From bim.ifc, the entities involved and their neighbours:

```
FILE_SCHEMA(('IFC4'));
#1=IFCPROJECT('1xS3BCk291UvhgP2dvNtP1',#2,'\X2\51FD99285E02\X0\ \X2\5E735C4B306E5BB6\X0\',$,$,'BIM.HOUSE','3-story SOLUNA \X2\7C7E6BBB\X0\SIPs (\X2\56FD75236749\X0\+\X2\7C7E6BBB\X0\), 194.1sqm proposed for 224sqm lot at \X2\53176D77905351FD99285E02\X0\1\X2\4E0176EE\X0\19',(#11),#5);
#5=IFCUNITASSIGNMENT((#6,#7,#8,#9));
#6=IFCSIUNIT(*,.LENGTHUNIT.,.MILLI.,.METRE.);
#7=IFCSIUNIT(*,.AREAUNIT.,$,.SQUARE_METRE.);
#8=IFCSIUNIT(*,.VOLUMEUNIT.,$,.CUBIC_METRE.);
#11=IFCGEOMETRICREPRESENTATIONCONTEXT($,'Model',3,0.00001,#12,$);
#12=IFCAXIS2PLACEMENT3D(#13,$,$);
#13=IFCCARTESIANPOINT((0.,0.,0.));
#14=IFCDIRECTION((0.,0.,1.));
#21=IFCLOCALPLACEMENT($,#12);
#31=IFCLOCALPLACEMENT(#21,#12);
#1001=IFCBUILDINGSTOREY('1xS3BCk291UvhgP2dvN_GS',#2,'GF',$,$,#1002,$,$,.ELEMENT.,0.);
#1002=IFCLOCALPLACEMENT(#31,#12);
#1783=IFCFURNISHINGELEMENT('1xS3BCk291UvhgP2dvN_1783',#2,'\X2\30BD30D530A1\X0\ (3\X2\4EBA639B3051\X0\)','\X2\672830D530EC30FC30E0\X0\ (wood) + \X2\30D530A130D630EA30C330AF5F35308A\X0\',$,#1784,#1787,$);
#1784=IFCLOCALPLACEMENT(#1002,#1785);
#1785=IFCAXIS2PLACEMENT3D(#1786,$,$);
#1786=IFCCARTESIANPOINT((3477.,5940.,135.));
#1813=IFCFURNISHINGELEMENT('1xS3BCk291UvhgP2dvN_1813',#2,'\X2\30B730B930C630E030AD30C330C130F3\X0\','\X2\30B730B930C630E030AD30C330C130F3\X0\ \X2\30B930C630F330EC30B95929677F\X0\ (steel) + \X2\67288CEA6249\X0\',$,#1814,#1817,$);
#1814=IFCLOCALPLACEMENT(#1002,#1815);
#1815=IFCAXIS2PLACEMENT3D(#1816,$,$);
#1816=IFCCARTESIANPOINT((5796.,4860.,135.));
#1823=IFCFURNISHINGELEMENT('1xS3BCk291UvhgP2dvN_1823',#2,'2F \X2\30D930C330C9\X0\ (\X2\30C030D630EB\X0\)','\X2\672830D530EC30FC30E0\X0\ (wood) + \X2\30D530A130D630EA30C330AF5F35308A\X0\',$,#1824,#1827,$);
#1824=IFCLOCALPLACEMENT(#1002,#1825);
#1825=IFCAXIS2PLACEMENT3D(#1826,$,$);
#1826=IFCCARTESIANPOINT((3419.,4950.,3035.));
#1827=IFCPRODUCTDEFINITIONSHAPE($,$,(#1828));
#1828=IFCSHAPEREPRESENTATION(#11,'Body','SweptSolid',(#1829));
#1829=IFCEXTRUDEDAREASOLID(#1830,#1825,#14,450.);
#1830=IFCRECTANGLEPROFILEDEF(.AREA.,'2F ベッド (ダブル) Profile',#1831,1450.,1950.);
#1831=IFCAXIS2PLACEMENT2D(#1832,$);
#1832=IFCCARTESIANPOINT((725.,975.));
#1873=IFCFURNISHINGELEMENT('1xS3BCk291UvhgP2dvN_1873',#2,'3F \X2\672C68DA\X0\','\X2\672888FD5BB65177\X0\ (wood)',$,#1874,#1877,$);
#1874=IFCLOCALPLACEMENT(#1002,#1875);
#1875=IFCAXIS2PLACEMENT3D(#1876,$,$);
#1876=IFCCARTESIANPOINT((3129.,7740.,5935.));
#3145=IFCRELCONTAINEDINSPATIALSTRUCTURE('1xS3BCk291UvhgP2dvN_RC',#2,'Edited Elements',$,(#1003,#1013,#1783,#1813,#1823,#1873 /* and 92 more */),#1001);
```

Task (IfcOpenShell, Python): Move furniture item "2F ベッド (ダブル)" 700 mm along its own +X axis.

```python
import ifcopenshell
import ifcopenshell.api.geometry
import ifcopenshell.util.placement

model = ifcopenshell.open("bim.ifc")

item = model.by_id(1823)
matrix = ifcopenshell.util.placement.get_local_placement(item.ObjectPlacement)
matrix[:3, 3] += matrix[:3, 0] * 700.0
ifcopenshell.api.geometry.edit_object_placement(model, product=item, matrix=matrix, is_si=False)

print(ifcopenshell.util.placement.get_local_placement(item.ObjectPlacement).round(3) + 0.0)

model.write("bim_rev.ifc")
```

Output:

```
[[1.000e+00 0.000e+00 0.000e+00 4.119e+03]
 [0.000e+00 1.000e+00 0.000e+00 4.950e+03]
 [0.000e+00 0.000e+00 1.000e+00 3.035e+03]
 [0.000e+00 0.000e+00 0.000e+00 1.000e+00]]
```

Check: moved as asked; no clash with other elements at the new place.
